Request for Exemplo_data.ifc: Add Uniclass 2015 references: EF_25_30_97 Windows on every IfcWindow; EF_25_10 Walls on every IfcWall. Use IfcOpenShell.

First a look at what the model holds.

```python
import ifcopenshell

model = ifcopenshell.open("Exemplo_data.ifc")
print(model.schema)
print("classifications:", [c.Name for c in model.by_type("IfcClassification")])
for ifc_class in ("IfcDoor", "IfcRoof", "IfcStair", "IfcWall", "IfcWindow"):
    print(ifc_class, len(model.by_type(ifc_class)))
```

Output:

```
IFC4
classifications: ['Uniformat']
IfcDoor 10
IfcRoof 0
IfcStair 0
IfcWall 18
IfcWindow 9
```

```python
import ifcopenshell
import ifcopenshell.api.classification

model = ifcopenshell.open("Exemplo_data.ifc")

system = ifcopenshell.api.classification.add_classification(model, classification="Uniclass 2015")

codes = {
    "IfcWindow": ("EF_25_30_97", "Windows"),
    "IfcWall": ("EF_25_10", "Walls"),
}
for ifc_class, (code, name) in codes.items():
    products = model.by_type(ifc_class)
    ifcopenshell.api.classification.add_reference(
        model, products=products, classification=system, identification=code, name=name
    )
    print(code, len(products))

model.write("Exemplo_data_edited.ifc")
```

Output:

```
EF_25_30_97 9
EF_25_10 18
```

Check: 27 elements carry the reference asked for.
